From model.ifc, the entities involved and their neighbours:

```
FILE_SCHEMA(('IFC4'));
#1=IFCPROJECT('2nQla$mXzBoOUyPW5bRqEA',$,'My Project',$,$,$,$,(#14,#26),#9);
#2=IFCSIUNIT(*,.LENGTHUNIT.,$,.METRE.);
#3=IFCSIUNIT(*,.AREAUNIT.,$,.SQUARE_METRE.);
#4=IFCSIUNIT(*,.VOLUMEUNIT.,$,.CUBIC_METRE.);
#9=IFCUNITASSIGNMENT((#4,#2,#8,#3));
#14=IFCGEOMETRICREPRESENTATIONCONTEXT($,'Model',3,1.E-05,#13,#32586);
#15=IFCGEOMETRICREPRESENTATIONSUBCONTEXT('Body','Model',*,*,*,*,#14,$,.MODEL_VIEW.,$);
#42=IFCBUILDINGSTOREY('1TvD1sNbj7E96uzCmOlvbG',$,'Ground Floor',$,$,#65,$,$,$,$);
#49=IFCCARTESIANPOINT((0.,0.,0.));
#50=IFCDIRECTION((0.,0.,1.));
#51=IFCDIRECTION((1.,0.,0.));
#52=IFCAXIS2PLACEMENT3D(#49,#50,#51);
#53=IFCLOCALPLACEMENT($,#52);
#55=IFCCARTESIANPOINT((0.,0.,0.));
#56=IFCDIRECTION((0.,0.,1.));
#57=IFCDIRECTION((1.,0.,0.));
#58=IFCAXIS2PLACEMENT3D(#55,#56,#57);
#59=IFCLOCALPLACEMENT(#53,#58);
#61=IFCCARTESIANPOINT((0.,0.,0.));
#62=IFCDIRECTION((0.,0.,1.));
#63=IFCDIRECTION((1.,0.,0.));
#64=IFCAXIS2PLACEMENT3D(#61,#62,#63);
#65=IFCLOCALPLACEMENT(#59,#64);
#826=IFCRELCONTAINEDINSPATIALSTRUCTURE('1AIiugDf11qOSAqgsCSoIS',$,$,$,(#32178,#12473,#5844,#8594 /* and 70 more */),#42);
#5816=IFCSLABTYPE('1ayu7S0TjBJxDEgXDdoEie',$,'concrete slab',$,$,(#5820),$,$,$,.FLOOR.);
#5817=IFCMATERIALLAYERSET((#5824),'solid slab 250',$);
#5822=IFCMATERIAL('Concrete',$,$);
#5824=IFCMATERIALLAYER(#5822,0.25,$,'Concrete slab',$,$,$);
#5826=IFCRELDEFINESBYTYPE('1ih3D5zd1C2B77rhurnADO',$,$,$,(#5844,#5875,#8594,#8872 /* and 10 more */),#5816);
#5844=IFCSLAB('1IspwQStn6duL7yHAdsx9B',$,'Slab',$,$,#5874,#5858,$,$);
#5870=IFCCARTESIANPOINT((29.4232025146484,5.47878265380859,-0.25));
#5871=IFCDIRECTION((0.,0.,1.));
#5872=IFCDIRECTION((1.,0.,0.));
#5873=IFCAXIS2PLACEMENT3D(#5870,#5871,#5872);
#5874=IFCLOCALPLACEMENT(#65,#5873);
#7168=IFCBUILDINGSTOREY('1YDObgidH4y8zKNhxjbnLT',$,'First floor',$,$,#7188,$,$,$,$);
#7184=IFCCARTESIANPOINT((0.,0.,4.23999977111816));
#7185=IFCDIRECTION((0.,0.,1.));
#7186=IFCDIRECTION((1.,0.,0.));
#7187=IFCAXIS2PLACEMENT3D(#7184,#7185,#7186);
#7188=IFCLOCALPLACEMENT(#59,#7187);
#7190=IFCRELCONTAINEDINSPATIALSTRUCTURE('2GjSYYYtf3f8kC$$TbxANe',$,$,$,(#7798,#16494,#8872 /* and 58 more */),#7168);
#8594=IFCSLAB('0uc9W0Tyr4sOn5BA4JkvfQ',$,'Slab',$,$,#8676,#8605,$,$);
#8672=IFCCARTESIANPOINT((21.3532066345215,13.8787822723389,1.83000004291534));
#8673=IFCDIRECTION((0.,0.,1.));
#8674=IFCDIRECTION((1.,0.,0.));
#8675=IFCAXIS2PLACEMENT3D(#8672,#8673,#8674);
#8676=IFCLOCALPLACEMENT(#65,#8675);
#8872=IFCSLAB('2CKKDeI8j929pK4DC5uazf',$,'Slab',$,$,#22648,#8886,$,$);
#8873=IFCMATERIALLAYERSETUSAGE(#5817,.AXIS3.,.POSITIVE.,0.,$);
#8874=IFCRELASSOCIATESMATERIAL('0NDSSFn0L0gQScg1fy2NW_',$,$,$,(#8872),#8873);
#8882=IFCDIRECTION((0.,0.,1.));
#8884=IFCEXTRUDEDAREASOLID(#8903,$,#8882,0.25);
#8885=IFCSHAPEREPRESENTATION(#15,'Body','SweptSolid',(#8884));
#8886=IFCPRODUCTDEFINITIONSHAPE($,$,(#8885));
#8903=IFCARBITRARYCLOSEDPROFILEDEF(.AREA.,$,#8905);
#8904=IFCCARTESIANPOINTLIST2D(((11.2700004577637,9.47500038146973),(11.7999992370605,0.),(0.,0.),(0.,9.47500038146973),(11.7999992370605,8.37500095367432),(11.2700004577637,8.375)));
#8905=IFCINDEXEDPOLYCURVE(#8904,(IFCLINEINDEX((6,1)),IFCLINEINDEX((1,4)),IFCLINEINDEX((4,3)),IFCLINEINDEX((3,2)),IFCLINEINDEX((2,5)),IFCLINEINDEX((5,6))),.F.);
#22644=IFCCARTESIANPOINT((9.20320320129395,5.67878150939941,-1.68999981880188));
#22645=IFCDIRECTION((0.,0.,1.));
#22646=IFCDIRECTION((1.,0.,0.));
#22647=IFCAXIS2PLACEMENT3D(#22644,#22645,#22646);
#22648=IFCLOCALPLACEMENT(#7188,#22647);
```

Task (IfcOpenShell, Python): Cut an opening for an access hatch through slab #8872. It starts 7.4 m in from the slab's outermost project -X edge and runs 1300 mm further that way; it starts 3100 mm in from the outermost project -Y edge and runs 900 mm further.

```python
import numpy as np
import ifcopenshell
import ifcopenshell.api.feature
import ifcopenshell.api.geometry
import ifcopenshell.api.root
import ifcopenshell.geom
import ifcopenshell.util.placement
import ifcopenshell.util.representation
import ifcopenshell.util.shape
import ifcopenshell.util.unit

model = ifcopenshell.open("model.ifc")
unit_scale = ifcopenshell.util.unit.calculate_unit_scale(model)
settings = ifcopenshell.geom.settings()


def volume(element):
    """Net volume in cubic metres, openings subtracted."""
    shape = ifcopenshell.geom.create_shape(settings, element)
    return ifcopenshell.util.shape.get_volume(shape.geometry)


slab = model.by_guid("2CKKDeI8j929pK4DC5uazf")
before = volume(slab)

# Extent in the slab's own axes, in metres. The edges named are its -X and -Y sides.
slab_shape = ifcopenshell.geom.create_shape(settings, slab)
vertices = ifcopenshell.util.shape.get_vertices(slab_shape.geometry)
x_min, y_min, bottom = vertices.min(axis=0)
top = vertices[:, 2].max()

opening = ifcopenshell.api.root.create_entity(model, ifc_class="IfcOpeningElement", name="Access hatch opening", predefined_type="OPENING")
context = ifcopenshell.util.representation.get_context(model, "Model", "Body", "MODEL_VIEW")
width, depth = 1.3, 0.9
outline = [(0.0, 0.0), (width, 0.0), (width, depth), (0.0, depth), (0.0, 0.0)]
# Overshoot both faces by 50 mm so the cut is clean.
shape = ifcopenshell.api.geometry.add_slab_representation(
    model, context=context, depth=top - bottom + 0.1, polyline=outline
)
ifcopenshell.api.geometry.assign_representation(model, product=opening, representation=shape)

matrix = ifcopenshell.util.placement.get_local_placement(slab.ObjectPlacement)
matrix[:, 3] = matrix @ np.append(np.array([x_min + 7.4, y_min + 3.1, bottom - 0.05]) / unit_scale, 1.0)
ifcopenshell.api.geometry.edit_object_placement(model, product=opening, matrix=matrix, is_si=False)
ifcopenshell.api.feature.add_feature(model, feature=opening, element=slab)

after = volume(slab)

print(f"slab volume {before:.3f} -> {after:.3f} m3")

model.write("model_v2.ifc")
```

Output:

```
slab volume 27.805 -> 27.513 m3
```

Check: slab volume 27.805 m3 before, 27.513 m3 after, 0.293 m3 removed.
